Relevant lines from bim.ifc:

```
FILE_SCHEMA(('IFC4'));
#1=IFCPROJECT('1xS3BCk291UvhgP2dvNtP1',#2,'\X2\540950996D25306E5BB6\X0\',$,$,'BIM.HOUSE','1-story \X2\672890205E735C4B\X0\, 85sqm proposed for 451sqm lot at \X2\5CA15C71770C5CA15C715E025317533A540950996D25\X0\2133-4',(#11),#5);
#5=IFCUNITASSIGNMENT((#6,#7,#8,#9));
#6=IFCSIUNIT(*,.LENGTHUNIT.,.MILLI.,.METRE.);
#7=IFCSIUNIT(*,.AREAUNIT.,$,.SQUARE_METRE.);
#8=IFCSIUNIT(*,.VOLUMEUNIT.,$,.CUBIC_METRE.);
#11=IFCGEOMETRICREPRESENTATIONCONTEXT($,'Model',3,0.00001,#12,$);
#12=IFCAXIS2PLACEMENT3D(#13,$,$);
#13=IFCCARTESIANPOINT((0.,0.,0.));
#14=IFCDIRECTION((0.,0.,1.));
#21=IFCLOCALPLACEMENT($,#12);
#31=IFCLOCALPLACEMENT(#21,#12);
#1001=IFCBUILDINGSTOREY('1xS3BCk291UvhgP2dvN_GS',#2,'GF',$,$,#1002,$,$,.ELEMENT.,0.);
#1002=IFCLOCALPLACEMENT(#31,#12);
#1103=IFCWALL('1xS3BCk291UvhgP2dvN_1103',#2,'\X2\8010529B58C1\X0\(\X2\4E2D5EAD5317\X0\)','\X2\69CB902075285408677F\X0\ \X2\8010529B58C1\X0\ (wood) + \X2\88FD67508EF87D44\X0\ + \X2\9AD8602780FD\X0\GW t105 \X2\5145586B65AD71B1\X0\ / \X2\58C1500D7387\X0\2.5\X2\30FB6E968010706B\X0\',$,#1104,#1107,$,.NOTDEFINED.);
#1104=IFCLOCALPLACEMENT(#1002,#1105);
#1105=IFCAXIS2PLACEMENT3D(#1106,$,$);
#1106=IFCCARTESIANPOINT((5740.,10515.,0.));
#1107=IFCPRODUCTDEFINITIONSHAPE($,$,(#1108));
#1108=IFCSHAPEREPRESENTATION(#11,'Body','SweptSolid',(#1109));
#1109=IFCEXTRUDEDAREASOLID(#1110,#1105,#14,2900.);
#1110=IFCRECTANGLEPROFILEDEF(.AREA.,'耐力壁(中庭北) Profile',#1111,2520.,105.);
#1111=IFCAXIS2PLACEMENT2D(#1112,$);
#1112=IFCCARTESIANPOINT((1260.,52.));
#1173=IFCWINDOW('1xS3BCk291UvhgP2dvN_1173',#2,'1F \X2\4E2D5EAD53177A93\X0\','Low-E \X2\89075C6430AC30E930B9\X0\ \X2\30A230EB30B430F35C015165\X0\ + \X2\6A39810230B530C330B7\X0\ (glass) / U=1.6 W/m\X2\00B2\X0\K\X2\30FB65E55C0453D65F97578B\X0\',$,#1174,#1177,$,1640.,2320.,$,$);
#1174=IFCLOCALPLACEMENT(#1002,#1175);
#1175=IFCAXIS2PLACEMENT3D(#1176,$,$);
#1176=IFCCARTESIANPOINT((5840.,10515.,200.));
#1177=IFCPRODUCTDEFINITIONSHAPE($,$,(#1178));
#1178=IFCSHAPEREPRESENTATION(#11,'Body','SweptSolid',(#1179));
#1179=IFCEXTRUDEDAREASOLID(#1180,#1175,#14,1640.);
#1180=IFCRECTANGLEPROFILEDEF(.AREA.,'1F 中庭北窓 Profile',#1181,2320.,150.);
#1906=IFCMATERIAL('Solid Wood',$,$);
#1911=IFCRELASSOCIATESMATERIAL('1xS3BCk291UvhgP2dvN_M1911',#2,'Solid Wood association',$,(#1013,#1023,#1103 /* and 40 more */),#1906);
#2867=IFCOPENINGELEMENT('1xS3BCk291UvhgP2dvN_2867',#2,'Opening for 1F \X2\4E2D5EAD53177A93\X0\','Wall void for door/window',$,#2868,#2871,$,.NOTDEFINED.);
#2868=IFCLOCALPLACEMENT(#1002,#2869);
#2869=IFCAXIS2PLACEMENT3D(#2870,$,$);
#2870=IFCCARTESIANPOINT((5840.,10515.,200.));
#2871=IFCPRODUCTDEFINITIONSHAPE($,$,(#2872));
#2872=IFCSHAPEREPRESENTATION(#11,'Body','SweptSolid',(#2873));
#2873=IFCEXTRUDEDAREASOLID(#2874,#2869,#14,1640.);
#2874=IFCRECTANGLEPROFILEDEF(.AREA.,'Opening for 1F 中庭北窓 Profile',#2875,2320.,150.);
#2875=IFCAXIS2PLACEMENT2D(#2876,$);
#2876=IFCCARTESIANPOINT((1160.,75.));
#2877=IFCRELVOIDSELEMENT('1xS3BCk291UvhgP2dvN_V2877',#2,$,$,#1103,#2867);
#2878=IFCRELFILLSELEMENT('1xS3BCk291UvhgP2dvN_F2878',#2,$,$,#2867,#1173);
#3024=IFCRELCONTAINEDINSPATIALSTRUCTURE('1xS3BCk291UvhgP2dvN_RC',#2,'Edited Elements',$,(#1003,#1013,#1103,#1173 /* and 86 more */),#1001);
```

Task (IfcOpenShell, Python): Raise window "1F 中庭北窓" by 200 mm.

```python
import numpy as np
import ifcopenshell
import ifcopenshell.api.geometry
import ifcopenshell.util.placement
import ifcopenshell.util.unit

model = ifcopenshell.open("bim.ifc")
unit_scale = ifcopenshell.util.unit.calculate_unit_scale(model)

window = model.by_id(1173)
opening = window.FillsVoids[0].RelatingOpeningElement
dz = 0.2 / unit_scale

shift = np.array([0.0, 0.0, dz])
# The window is not placed relative to its opening, so move both.
for product in (opening, window):
    matrix = ifcopenshell.util.placement.get_local_placement(product.ObjectPlacement)
    matrix[:3, 3] += shift
    ifcopenshell.api.geometry.edit_object_placement(model, product=product, matrix=matrix, is_si=False)

print(f"moved by {dz * unit_scale:+.3f} m")

model.write("bim_v2.ifc")
```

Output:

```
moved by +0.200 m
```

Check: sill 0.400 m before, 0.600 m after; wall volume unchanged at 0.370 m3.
